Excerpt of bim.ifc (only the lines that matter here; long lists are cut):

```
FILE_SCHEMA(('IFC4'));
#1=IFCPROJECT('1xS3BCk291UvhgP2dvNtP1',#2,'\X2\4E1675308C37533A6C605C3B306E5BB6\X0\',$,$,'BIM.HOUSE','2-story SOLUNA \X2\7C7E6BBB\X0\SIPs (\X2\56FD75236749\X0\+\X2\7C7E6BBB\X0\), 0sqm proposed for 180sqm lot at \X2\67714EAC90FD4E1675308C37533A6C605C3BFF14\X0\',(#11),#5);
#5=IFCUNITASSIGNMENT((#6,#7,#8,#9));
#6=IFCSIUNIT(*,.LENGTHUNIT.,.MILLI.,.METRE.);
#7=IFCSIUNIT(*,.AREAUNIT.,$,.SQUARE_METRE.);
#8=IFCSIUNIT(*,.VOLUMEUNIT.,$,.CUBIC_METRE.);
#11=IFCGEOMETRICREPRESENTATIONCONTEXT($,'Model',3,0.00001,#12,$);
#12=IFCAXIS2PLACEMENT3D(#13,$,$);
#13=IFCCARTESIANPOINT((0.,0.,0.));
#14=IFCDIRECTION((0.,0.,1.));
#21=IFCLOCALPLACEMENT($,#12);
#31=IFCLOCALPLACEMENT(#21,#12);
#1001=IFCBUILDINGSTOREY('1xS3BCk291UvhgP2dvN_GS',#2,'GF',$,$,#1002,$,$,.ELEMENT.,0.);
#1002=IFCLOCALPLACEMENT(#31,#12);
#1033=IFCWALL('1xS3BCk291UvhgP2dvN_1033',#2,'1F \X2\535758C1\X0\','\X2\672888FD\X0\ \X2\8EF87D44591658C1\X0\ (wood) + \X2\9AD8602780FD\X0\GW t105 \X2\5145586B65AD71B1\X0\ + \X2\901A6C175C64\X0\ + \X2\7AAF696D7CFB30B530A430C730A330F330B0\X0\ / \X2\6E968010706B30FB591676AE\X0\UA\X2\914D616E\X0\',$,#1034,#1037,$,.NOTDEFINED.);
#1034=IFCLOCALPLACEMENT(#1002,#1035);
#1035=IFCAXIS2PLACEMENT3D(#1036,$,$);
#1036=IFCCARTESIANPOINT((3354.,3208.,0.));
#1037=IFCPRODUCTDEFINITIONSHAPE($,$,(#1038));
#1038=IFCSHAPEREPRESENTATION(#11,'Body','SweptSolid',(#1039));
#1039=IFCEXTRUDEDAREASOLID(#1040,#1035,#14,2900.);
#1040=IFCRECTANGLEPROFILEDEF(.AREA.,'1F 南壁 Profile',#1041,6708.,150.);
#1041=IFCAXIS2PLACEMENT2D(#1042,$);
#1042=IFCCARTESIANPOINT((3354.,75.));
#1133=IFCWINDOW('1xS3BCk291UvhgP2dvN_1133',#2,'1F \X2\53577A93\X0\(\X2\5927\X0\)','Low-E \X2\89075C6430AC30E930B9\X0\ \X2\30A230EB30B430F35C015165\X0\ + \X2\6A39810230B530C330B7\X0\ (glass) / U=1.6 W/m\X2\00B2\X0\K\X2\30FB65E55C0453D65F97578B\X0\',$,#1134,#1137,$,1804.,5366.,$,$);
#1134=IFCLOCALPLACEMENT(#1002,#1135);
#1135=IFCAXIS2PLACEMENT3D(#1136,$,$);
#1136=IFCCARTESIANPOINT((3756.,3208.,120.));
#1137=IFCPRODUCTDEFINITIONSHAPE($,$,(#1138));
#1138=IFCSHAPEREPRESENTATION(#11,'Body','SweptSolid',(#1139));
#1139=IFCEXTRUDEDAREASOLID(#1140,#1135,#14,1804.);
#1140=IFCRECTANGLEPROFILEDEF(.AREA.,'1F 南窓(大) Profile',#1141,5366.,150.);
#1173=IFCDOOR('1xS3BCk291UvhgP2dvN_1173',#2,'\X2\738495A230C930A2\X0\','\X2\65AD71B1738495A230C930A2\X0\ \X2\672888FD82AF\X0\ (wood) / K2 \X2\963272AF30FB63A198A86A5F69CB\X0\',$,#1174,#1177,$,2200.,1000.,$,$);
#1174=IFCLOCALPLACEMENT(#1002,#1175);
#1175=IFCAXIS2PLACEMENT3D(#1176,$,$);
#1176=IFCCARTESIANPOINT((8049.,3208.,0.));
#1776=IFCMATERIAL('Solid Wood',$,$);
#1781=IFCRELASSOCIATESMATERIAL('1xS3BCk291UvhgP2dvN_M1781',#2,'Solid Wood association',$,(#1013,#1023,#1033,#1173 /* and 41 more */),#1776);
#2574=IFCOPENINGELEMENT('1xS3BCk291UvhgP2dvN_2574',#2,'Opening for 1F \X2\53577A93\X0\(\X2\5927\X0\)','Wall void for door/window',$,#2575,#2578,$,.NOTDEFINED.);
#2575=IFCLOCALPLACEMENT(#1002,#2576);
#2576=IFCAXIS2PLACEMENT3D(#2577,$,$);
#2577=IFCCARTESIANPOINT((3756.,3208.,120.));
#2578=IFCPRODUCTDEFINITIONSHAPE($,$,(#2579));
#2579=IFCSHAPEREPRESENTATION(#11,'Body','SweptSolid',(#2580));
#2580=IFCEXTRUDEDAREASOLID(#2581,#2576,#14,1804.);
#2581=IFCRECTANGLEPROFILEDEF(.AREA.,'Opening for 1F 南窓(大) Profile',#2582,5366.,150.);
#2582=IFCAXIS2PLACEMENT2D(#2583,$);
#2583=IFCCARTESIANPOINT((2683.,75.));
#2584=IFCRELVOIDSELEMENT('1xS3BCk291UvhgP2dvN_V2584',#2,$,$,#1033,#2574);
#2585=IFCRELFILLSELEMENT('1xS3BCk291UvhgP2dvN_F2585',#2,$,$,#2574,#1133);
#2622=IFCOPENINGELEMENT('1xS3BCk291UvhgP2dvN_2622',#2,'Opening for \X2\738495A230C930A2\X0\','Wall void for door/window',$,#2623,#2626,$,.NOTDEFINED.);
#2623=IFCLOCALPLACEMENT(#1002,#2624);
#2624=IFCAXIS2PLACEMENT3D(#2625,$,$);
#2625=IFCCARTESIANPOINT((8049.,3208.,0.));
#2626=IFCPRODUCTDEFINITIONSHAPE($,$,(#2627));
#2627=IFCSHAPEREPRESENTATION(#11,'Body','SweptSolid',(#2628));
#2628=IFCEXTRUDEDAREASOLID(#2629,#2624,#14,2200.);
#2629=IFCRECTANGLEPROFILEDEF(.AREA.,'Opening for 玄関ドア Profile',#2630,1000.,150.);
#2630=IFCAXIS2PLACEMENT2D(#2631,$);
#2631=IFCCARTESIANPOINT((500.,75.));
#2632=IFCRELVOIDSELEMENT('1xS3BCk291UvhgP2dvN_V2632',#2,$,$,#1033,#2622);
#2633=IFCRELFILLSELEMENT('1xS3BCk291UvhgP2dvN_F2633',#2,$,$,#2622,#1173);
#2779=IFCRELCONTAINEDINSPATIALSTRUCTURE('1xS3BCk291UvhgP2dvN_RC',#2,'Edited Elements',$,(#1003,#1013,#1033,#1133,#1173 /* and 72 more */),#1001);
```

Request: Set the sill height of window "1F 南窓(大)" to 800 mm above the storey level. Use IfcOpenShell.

```python
import numpy as np
import ifcopenshell
import ifcopenshell.api.geometry
import ifcopenshell.geom
import ifcopenshell.util.element
import ifcopenshell.util.placement
import ifcopenshell.util.shape
import ifcopenshell.util.unit

model = ifcopenshell.open("bim.ifc")
unit_scale = ifcopenshell.util.unit.calculate_unit_scale(model)

window = model.by_id(1133)
opening = window.FillsVoids[0].RelatingOpeningElement
storey = ifcopenshell.util.element.get_container(window, ifc_class="IfcBuildingStorey")
level = ifcopenshell.util.placement.get_local_placement(storey.ObjectPlacement)[2, 3]

# The opening's origin need not be at the sill, so measure its lowest point.
shape = ifcopenshell.geom.create_shape(ifcopenshell.geom.settings(), opening)
bottom = ifcopenshell.util.shape.get_shape_bottom_elevation(shape, shape.geometry) / unit_scale
dz = level + 0.8 / unit_scale - bottom

shift = np.array([0.0, 0.0, dz])
# The window is not placed relative to its opening, so move both.
for product in (opening, window):
    matrix = ifcopenshell.util.placement.get_local_placement(product.ObjectPlacement)
    matrix[:3, 3] += shift
    ifcopenshell.api.geometry.edit_object_placement(model, product=product, matrix=matrix, is_si=False)

print(f"moved by {dz * unit_scale:+.3f} m")

model.write("bim_rev.ifc")
```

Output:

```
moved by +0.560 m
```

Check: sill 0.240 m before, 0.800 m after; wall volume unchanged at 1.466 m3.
